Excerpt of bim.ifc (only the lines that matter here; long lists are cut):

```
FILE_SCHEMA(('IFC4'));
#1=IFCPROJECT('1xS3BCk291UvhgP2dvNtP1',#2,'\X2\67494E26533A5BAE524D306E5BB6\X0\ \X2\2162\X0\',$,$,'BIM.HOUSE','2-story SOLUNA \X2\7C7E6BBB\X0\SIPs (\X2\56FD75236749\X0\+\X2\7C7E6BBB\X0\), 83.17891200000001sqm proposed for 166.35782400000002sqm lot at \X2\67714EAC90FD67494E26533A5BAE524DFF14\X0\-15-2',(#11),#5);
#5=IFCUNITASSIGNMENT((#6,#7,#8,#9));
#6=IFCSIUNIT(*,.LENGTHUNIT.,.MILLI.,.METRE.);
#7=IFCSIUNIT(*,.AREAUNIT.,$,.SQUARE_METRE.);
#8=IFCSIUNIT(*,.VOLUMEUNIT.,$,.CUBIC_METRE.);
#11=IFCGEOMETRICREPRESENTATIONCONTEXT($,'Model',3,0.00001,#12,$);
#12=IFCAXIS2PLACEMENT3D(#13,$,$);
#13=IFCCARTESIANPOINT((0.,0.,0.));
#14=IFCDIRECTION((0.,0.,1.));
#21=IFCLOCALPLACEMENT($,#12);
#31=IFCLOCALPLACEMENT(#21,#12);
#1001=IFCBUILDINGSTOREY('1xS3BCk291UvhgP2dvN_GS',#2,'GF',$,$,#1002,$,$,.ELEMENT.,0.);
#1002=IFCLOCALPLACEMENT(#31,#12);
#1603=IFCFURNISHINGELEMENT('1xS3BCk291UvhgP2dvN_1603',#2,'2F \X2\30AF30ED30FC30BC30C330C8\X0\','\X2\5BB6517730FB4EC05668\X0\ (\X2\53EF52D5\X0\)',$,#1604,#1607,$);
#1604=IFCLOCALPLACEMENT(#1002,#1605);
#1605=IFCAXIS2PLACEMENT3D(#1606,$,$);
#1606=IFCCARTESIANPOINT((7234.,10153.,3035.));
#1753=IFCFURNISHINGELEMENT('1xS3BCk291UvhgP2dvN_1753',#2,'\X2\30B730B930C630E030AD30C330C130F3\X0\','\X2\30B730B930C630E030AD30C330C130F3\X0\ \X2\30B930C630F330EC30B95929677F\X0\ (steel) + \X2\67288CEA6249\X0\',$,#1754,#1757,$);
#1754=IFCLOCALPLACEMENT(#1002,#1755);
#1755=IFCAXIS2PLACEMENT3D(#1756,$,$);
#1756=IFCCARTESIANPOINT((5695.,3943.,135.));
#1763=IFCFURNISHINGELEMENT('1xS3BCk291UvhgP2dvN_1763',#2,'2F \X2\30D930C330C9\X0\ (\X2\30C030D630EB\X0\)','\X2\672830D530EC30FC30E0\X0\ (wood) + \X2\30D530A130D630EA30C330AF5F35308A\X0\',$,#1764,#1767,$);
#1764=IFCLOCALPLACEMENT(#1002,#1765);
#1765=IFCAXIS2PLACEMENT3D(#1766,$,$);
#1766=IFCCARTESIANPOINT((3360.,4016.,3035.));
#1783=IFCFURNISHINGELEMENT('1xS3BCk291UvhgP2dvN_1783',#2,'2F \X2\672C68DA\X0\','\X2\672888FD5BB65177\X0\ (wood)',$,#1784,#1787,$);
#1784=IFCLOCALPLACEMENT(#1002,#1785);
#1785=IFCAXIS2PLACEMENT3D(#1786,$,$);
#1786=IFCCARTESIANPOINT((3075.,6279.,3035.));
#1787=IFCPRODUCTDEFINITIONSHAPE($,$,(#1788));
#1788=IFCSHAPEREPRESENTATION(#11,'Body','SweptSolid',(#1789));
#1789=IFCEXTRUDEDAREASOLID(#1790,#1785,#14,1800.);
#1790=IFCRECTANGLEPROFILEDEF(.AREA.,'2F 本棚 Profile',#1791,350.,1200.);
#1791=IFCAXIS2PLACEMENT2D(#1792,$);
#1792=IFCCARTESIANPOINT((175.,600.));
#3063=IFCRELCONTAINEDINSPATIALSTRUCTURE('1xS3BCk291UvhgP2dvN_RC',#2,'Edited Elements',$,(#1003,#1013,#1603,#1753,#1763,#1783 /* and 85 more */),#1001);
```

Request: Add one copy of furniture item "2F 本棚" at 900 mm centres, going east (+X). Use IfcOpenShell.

```python
import numpy as np
import ifcopenshell
import ifcopenshell.api.geometry
import ifcopenshell.api.root
import ifcopenshell.util.element
import ifcopenshell.util.placement

model = ifcopenshell.open("bim.ifc")


def reuse_history(source, copy):
    """copy_class also copies each property set's owner history, people and application; keep the originals."""
    for rel in copy.IsDefinedBy:
        if rel.is_a("IfcRelDefinesByProperties") and (history := rel.RelatingPropertyDefinition.OwnerHistory):
            rel.RelatingPropertyDefinition.OwnerHistory = source.OwnerHistory
            ifcopenshell.util.element.remove_deep2(model, history)


source = model.by_id(1783)
base = ifcopenshell.util.placement.get_local_placement(source.ObjectPlacement)
step = np.array([1.0, 0.0, 0.0]) * 900.0

for i in range(1, 2):
    copy = ifcopenshell.api.root.copy_class(model, product=source)
    copy.Representation = ifcopenshell.util.element.copy_deep(
        model, source.Representation, exclude=["IfcGeometricRepresentationContext", "IfcRepresentationMap"]
    )
    reuse_history(source, copy)
    matrix = base.copy()
    matrix[:3, 3] += i * step
    print("added at", matrix[:3, 3].round(3) + 0.0)
    ifcopenshell.api.geometry.edit_object_placement(model, product=copy, matrix=matrix, is_si=False)

model.write("bim-out.ifc")
```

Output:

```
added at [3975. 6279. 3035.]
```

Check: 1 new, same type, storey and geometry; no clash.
